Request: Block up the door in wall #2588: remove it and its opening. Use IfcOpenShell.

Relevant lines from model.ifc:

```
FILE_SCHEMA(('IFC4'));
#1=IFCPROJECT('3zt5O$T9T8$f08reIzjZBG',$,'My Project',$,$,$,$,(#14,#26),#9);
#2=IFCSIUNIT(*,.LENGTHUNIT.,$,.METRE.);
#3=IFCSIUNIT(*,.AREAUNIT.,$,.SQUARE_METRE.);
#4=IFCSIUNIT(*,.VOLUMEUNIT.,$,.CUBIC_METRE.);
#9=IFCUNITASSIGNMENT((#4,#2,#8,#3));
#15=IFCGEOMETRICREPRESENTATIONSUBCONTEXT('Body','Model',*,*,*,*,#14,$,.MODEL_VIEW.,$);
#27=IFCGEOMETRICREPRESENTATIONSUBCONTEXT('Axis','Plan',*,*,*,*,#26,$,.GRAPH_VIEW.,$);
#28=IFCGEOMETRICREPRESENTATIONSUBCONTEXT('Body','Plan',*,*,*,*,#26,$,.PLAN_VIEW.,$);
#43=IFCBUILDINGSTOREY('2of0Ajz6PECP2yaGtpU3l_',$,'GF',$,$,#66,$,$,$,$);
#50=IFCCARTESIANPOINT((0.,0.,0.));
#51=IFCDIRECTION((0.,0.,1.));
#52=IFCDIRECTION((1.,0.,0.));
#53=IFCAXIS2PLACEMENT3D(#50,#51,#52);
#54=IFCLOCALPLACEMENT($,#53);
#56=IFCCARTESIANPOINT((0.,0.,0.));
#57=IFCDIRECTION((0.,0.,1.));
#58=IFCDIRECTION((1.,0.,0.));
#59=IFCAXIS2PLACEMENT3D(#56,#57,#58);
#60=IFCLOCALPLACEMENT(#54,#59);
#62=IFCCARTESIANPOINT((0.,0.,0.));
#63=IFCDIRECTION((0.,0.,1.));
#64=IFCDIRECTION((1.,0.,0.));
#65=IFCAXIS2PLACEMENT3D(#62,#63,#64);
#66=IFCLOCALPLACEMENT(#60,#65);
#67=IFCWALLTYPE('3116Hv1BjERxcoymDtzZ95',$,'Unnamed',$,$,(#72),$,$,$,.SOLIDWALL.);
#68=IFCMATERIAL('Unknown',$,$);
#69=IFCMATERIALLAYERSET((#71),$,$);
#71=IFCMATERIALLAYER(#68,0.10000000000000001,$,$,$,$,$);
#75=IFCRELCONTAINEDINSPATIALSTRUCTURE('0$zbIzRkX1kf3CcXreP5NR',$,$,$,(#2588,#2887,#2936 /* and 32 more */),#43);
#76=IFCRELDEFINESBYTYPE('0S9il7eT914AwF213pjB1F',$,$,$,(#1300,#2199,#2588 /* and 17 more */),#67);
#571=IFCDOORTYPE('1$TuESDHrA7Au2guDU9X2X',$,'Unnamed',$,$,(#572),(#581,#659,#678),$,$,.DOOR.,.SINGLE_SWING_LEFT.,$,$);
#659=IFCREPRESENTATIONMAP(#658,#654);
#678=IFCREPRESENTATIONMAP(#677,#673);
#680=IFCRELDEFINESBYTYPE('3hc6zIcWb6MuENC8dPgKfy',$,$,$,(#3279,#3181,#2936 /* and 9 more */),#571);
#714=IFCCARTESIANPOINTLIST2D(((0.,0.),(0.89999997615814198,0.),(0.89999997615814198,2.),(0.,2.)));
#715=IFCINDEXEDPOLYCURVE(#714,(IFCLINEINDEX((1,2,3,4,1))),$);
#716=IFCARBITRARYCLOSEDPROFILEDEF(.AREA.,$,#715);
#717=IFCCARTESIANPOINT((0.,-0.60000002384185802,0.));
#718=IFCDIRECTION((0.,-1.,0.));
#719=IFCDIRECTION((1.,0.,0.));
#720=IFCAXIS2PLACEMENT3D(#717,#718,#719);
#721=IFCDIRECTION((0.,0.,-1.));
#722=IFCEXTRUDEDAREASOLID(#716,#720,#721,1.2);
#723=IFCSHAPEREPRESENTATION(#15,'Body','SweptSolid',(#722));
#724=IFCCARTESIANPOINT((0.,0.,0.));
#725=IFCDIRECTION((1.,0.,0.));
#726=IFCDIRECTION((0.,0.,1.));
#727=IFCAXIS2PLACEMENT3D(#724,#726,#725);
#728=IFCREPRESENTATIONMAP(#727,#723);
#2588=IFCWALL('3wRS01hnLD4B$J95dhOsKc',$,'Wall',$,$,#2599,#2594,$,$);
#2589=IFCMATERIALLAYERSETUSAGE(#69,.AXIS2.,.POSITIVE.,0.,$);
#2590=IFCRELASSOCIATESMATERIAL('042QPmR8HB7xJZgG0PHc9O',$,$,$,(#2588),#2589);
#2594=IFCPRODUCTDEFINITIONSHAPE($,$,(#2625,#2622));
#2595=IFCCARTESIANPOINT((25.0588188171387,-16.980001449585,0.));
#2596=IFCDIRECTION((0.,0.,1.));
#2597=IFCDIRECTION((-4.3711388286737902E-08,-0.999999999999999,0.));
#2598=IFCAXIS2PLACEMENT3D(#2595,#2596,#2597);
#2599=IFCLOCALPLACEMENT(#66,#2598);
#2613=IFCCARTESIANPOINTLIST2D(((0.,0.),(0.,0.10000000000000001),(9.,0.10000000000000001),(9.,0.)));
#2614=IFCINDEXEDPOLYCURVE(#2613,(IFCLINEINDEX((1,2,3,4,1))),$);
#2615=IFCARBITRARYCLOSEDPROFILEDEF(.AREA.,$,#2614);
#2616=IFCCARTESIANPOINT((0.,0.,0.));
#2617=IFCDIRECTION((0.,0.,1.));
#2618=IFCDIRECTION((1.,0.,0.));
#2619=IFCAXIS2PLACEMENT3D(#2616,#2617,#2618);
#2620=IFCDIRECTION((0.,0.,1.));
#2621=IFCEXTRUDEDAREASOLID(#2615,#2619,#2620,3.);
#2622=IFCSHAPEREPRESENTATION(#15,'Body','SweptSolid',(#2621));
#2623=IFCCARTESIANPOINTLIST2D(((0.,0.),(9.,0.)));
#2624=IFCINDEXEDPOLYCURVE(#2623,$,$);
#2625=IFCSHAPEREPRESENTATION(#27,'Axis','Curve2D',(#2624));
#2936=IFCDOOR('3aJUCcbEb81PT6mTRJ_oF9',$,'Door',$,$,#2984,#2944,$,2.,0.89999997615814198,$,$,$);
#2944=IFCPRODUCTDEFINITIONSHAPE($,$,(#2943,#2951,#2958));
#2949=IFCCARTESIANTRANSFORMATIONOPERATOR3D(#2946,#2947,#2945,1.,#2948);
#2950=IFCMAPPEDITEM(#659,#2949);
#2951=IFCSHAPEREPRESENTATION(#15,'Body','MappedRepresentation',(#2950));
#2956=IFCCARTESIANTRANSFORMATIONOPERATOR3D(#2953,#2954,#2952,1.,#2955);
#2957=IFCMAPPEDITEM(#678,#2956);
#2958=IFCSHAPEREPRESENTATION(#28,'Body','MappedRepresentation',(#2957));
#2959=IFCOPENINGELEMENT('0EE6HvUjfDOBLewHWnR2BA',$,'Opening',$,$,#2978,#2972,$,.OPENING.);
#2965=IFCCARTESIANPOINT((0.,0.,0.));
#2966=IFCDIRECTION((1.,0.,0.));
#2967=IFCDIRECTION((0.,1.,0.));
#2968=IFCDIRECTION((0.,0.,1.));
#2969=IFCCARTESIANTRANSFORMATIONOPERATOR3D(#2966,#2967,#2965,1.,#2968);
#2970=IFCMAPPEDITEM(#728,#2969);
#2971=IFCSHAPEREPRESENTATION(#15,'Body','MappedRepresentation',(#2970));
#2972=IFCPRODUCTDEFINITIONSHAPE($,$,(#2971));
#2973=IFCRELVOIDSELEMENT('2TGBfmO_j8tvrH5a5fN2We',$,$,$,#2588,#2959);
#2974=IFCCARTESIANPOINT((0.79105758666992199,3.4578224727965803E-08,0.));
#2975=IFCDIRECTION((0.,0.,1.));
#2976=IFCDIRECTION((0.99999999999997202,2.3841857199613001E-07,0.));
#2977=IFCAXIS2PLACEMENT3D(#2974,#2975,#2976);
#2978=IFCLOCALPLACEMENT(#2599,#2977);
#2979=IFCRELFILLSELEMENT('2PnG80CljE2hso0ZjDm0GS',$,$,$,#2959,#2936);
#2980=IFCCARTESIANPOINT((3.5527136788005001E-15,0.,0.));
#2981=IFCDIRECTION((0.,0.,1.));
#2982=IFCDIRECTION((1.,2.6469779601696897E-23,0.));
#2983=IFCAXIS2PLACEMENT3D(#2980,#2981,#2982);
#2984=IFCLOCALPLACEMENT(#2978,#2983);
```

```python
import ifcopenshell
import ifcopenshell.api.feature
import ifcopenshell.api.root
import ifcopenshell.geom
import ifcopenshell.util.shape

model = ifcopenshell.open("model.ifc")
settings = ifcopenshell.geom.settings()


def volume(element):
    """Net volume in cubic metres, openings subtracted."""
    shape = ifcopenshell.geom.create_shape(settings, element)
    return ifcopenshell.util.shape.get_volume(shape.geometry)


door = model.by_id(2936)
opening = door.FillsVoids[0].RelatingOpeningElement
wall = opening.VoidsElements[0].RelatingBuildingElement
before = volume(wall)

ifcopenshell.api.root.remove_product(model, product=door)
ifcopenshell.api.feature.remove_feature(model, feature=opening)

after = volume(wall)

print(f"wall volume {before:.3f} -> {after:.3f} m3")

model.write("model_updated.ifc")
```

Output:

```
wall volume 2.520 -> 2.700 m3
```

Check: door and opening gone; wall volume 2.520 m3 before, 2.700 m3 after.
